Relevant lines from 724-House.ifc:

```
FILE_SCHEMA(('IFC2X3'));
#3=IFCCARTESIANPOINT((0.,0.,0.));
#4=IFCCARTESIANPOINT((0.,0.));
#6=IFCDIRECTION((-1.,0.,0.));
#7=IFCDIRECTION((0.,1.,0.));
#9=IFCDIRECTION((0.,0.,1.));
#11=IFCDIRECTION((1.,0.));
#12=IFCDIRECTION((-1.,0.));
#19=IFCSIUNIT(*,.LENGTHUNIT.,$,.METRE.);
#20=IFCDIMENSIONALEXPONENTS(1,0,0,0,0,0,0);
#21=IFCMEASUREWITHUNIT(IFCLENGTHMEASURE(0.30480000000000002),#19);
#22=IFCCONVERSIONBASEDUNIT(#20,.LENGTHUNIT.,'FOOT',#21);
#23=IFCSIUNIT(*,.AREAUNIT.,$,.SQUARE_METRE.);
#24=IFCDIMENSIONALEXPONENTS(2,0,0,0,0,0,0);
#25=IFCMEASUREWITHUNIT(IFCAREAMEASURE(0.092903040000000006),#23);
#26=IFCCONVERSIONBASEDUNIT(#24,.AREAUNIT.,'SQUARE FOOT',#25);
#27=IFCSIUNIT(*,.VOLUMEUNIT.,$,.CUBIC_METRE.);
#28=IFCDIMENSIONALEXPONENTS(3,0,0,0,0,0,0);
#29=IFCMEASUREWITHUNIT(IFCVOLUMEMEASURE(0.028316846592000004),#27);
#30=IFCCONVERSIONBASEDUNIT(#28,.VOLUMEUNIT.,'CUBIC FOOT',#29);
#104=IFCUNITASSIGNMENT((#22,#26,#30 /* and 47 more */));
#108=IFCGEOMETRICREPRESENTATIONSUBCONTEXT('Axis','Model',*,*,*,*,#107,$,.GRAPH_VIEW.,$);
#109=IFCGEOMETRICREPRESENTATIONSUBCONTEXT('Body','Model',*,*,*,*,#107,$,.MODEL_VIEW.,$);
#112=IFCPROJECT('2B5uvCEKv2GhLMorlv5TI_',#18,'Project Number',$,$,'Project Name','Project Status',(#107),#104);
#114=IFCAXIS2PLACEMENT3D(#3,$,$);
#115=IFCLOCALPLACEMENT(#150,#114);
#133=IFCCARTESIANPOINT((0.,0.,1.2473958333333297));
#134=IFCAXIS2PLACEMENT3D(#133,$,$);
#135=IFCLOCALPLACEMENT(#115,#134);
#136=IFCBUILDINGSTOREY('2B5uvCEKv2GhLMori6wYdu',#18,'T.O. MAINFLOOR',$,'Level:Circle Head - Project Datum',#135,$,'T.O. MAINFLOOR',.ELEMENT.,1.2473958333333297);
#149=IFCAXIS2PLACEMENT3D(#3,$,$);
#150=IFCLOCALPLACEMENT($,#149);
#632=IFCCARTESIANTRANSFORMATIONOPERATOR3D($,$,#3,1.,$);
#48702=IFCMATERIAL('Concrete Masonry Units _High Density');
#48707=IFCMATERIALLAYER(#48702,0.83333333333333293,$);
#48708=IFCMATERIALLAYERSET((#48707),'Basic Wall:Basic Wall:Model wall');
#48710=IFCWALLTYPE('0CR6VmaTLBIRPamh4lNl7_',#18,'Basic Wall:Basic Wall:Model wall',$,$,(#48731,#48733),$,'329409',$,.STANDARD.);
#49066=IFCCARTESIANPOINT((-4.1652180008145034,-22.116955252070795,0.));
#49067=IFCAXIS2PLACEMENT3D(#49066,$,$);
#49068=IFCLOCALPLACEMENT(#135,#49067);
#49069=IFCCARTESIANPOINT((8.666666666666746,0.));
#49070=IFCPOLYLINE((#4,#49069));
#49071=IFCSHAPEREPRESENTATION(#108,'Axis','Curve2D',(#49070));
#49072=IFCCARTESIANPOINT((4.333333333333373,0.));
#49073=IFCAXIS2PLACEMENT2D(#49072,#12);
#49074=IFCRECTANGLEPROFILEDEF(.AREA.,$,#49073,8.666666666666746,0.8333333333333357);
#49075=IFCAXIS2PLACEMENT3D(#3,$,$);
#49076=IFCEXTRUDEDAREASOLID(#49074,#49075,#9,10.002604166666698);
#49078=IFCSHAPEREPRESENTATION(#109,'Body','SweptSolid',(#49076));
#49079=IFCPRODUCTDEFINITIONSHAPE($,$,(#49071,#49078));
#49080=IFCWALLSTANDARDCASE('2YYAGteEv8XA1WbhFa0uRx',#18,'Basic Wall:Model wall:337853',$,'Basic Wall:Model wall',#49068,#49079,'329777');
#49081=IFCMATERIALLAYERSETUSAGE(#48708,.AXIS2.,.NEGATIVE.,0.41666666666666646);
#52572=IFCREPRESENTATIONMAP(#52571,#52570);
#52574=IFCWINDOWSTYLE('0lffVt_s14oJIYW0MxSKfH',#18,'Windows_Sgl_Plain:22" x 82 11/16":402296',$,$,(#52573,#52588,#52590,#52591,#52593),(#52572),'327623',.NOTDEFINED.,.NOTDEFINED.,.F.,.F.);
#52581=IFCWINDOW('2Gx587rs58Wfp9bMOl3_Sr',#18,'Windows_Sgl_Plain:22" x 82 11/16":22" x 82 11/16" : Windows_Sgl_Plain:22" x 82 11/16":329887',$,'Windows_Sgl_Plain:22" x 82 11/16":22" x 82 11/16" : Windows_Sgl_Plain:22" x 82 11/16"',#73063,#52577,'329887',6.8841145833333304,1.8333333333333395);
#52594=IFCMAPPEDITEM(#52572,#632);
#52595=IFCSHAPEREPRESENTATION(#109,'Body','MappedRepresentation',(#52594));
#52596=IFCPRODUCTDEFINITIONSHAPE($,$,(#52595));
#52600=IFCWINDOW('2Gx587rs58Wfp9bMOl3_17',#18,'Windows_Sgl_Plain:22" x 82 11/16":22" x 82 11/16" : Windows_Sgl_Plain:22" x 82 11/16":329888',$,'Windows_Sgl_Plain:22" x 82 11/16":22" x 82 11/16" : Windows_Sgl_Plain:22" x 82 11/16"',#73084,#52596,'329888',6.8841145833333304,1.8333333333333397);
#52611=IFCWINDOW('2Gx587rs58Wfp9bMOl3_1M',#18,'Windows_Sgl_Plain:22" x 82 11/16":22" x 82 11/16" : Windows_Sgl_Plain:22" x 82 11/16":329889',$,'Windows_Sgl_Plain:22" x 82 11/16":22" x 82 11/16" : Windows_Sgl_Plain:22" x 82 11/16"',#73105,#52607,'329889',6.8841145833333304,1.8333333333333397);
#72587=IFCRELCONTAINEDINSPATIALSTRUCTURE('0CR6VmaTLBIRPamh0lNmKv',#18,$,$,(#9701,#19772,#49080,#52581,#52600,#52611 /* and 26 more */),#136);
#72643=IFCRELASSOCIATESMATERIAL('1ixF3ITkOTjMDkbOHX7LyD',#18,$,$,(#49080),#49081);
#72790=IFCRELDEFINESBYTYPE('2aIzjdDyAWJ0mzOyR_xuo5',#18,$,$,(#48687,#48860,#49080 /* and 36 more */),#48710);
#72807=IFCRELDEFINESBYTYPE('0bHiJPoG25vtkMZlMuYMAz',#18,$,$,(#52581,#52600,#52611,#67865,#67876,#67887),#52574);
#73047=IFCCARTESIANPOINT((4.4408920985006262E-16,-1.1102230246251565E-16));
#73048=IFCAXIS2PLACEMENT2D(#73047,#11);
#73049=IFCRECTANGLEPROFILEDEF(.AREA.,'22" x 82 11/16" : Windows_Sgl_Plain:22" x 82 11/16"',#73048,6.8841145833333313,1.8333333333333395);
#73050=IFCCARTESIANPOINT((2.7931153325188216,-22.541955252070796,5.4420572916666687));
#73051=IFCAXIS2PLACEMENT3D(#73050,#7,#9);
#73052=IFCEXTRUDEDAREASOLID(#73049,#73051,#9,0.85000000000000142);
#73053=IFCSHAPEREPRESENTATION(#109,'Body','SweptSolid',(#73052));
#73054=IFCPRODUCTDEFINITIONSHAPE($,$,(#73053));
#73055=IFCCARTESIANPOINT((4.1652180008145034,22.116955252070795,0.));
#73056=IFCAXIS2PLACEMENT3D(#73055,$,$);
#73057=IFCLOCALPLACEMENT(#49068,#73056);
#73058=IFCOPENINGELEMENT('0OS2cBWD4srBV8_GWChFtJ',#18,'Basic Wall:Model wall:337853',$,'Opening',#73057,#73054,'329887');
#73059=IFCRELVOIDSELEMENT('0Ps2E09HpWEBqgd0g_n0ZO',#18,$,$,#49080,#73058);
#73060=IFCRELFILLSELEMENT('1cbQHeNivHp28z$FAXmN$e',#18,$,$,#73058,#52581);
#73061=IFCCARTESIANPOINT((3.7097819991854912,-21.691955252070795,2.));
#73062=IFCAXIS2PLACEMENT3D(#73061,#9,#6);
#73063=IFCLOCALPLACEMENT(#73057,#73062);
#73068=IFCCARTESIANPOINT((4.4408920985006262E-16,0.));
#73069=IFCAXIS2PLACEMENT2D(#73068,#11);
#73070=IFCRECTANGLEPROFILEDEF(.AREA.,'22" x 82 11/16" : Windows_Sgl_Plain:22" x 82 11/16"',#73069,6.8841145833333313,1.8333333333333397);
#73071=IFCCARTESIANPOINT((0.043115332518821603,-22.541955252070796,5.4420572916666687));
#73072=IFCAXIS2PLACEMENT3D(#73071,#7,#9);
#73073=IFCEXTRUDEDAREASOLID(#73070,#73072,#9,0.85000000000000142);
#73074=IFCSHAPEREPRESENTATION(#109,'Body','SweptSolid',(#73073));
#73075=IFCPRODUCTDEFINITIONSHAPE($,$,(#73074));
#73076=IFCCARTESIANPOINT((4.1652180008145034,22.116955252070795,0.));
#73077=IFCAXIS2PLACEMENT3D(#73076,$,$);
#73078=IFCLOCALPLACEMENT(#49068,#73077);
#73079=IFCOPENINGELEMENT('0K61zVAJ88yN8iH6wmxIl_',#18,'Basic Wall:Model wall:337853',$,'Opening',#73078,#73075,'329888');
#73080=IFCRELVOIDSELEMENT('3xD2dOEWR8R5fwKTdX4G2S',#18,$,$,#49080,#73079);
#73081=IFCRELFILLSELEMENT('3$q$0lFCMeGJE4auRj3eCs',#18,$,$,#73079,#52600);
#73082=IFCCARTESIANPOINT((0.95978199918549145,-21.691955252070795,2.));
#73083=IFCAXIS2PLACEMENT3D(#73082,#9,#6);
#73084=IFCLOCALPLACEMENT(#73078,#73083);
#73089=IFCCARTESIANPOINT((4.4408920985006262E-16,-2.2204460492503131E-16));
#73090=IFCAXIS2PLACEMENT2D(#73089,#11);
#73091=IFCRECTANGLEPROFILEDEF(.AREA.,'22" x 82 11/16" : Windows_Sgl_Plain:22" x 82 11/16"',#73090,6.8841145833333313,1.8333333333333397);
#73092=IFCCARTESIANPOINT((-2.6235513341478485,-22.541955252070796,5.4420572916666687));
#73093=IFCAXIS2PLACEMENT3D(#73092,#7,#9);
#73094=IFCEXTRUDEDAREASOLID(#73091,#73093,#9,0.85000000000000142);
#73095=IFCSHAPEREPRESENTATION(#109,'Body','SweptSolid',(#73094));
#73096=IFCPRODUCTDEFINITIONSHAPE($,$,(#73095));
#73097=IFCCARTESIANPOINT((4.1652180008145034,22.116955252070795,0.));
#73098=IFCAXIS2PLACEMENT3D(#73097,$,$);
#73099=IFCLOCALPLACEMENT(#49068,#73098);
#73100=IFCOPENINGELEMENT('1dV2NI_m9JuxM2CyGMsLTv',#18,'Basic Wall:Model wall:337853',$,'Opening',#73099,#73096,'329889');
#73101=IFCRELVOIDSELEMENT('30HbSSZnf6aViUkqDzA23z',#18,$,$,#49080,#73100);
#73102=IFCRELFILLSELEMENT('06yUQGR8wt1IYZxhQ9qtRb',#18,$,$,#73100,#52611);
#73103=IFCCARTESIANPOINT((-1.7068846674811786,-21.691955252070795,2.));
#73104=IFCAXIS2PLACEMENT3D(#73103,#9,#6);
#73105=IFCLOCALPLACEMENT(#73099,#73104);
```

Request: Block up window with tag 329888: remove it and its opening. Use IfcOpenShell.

```python
import ifcopenshell
import ifcopenshell.api.feature
import ifcopenshell.api.root
import ifcopenshell.geom
import ifcopenshell.util.shape

model = ifcopenshell.open("724-House.ifc")
settings = ifcopenshell.geom.settings()


def volume(element):
    """Net volume in cubic metres, openings subtracted."""
    shape = ifcopenshell.geom.create_shape(settings, element)
    return ifcopenshell.util.shape.get_volume(shape.geometry)


window = model.by_id(52600)
opening = window.FillsVoids[0].RelatingOpeningElement
wall = opening.VoidsElements[0].RelatingBuildingElement
before = volume(wall)

ifcopenshell.api.root.remove_product(model, product=window)
ifcopenshell.api.feature.remove_feature(model, feature=opening)

after = volume(wall)

print(f"wall volume {before:.3f} -> {after:.3f} m3")

model.write("724-House_edited.ifc")
```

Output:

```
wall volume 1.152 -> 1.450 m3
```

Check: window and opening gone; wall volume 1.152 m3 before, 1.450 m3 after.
